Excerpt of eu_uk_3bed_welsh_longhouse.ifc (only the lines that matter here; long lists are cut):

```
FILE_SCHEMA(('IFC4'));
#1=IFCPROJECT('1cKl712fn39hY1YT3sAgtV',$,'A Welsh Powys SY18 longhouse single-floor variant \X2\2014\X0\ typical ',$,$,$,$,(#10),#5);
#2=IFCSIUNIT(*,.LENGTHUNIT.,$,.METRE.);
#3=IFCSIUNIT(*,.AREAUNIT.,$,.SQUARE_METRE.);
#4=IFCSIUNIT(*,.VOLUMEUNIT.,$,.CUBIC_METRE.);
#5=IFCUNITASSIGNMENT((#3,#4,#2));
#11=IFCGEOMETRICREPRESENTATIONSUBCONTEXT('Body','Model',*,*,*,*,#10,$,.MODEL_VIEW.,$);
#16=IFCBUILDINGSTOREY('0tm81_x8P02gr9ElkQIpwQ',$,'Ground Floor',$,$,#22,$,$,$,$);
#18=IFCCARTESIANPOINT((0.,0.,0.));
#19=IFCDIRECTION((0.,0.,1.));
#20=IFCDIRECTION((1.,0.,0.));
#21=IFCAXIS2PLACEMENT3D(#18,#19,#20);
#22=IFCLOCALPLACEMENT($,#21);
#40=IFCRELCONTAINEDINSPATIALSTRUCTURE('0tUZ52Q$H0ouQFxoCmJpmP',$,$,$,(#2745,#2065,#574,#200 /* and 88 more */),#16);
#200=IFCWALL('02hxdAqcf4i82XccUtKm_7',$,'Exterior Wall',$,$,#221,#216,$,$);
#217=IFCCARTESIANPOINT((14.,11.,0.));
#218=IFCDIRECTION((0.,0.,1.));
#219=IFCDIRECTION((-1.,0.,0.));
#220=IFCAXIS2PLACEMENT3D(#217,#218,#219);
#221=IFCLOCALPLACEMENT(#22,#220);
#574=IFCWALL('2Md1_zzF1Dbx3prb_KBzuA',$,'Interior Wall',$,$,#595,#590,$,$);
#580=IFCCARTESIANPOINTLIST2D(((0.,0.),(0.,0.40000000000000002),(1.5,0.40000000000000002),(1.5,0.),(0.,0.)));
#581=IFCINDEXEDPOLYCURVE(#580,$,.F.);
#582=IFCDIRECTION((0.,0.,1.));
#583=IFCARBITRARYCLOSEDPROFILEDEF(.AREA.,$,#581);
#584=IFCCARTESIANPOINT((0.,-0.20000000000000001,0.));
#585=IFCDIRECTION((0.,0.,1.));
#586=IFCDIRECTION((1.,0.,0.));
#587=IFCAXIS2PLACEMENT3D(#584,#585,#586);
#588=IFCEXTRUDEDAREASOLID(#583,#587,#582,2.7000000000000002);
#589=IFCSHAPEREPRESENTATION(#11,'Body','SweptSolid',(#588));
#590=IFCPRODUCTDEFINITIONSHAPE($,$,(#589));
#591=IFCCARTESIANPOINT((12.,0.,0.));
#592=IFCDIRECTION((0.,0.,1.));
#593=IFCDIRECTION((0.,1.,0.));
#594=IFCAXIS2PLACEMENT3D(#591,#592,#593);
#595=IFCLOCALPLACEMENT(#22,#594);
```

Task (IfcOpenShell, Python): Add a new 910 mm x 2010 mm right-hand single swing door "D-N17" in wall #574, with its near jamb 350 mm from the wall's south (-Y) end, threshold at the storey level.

```python
import numpy as np
import ifcopenshell
import ifcopenshell.api.feature
import ifcopenshell.api.geometry
import ifcopenshell.api.root
import ifcopenshell.api.spatial
import ifcopenshell.geom
import ifcopenshell.util.element
import ifcopenshell.util.placement
import ifcopenshell.util.representation
import ifcopenshell.util.shape
import ifcopenshell.util.unit

model = ifcopenshell.open("eu_uk_3bed_welsh_longhouse.ifc")
unit_scale = ifcopenshell.util.unit.calculate_unit_scale(model)
settings = ifcopenshell.geom.settings()


def volume(element):
    """Net volume in cubic metres, openings subtracted."""
    shape = ifcopenshell.geom.create_shape(settings, element)
    return ifcopenshell.util.shape.get_volume(shape.geometry)


wall = model.by_guid("2Md1_zzF1Dbx3prb_KBzuA")
storey = ifcopenshell.util.element.get_container(wall, ifc_class="IfcBuildingStorey")
context = ifcopenshell.util.representation.get_context(model, "Model", "Body", "MODEL_VIEW")
before = volume(wall)

width, height, from_end, sill = 0.91, 2.01, 0.35, 0.0  # metres

# The wall runs along its own X axis, and the end named is its -X end.
wall_shape = ifcopenshell.geom.create_shape(settings, wall)
x, y, z = ifcopenshell.util.shape.get_vertices(wall_shape.geometry).T
start = x.min() + from_end
face, thickness = float(y.min()), float(y.max() - y.min())
wall_matrix = ifcopenshell.util.placement.get_local_placement(wall.ObjectPlacement)
level = ifcopenshell.util.placement.get_local_placement(storey.ObjectPlacement)[2, 3]


def in_wall(x, y):
    """Placement at x, y metres in the wall's axes, at sill height."""
    matrix = wall_matrix.copy()
    matrix[:, 3] = wall_matrix @ np.array([x / unit_scale, y / unit_scale, 0.0, 1.0])
    matrix[2, 3] = level + sill / unit_scale
    return matrix


# Opening: a box that overshoots both wall faces by 50 mm.
opening = ifcopenshell.api.root.create_entity(model, ifc_class="IfcOpeningElement", predefined_type="OPENING")
box = ifcopenshell.api.geometry.add_wall_representation(
    model, context=context, length=width, height=height, thickness=thickness + 0.1
)
ifcopenshell.api.geometry.assign_representation(model, product=opening, representation=box)
ifcopenshell.api.geometry.edit_object_placement(model, product=opening, matrix=in_wall(start, face - 0.05), is_si=False)
ifcopenshell.api.feature.add_feature(model, feature=opening, element=wall)

door = ifcopenshell.api.root.create_entity(model, ifc_class="IfcDoor", name="D-N17", predefined_type="DOOR")
door.OverallWidth, door.OverallHeight = width / unit_scale, height / unit_scale
door.OperationType = "SINGLE_SWING_RIGHT"
body = ifcopenshell.api.geometry.add_door_representation(
    model,
    context=context,
    overall_width=door.OverallWidth,
    overall_height=door.OverallHeight,
    operation_type="SINGLE_SWING_RIGHT",
    lining_properties={"LiningDepth": thickness / unit_scale, "ThresholdDepth": thickness / unit_scale},
)
ifcopenshell.api.geometry.assign_representation(model, product=door, representation=body)
ifcopenshell.api.spatial.assign_container(model, products=[door], relating_structure=storey)
ifcopenshell.api.feature.add_filling(model, opening=opening, element=door)

# The lining spans the wall, so the door starts at the wall face.
ifcopenshell.api.geometry.edit_object_placement(model, product=door, matrix=in_wall(start, face), is_si=False)

after = volume(wall)

print(f"wall volume {before:.3f} -> {after:.3f} m3")

model.write("eu_uk_3bed_welsh_longhouse_rev.ifc")
```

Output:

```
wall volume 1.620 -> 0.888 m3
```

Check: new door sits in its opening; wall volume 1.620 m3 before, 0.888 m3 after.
